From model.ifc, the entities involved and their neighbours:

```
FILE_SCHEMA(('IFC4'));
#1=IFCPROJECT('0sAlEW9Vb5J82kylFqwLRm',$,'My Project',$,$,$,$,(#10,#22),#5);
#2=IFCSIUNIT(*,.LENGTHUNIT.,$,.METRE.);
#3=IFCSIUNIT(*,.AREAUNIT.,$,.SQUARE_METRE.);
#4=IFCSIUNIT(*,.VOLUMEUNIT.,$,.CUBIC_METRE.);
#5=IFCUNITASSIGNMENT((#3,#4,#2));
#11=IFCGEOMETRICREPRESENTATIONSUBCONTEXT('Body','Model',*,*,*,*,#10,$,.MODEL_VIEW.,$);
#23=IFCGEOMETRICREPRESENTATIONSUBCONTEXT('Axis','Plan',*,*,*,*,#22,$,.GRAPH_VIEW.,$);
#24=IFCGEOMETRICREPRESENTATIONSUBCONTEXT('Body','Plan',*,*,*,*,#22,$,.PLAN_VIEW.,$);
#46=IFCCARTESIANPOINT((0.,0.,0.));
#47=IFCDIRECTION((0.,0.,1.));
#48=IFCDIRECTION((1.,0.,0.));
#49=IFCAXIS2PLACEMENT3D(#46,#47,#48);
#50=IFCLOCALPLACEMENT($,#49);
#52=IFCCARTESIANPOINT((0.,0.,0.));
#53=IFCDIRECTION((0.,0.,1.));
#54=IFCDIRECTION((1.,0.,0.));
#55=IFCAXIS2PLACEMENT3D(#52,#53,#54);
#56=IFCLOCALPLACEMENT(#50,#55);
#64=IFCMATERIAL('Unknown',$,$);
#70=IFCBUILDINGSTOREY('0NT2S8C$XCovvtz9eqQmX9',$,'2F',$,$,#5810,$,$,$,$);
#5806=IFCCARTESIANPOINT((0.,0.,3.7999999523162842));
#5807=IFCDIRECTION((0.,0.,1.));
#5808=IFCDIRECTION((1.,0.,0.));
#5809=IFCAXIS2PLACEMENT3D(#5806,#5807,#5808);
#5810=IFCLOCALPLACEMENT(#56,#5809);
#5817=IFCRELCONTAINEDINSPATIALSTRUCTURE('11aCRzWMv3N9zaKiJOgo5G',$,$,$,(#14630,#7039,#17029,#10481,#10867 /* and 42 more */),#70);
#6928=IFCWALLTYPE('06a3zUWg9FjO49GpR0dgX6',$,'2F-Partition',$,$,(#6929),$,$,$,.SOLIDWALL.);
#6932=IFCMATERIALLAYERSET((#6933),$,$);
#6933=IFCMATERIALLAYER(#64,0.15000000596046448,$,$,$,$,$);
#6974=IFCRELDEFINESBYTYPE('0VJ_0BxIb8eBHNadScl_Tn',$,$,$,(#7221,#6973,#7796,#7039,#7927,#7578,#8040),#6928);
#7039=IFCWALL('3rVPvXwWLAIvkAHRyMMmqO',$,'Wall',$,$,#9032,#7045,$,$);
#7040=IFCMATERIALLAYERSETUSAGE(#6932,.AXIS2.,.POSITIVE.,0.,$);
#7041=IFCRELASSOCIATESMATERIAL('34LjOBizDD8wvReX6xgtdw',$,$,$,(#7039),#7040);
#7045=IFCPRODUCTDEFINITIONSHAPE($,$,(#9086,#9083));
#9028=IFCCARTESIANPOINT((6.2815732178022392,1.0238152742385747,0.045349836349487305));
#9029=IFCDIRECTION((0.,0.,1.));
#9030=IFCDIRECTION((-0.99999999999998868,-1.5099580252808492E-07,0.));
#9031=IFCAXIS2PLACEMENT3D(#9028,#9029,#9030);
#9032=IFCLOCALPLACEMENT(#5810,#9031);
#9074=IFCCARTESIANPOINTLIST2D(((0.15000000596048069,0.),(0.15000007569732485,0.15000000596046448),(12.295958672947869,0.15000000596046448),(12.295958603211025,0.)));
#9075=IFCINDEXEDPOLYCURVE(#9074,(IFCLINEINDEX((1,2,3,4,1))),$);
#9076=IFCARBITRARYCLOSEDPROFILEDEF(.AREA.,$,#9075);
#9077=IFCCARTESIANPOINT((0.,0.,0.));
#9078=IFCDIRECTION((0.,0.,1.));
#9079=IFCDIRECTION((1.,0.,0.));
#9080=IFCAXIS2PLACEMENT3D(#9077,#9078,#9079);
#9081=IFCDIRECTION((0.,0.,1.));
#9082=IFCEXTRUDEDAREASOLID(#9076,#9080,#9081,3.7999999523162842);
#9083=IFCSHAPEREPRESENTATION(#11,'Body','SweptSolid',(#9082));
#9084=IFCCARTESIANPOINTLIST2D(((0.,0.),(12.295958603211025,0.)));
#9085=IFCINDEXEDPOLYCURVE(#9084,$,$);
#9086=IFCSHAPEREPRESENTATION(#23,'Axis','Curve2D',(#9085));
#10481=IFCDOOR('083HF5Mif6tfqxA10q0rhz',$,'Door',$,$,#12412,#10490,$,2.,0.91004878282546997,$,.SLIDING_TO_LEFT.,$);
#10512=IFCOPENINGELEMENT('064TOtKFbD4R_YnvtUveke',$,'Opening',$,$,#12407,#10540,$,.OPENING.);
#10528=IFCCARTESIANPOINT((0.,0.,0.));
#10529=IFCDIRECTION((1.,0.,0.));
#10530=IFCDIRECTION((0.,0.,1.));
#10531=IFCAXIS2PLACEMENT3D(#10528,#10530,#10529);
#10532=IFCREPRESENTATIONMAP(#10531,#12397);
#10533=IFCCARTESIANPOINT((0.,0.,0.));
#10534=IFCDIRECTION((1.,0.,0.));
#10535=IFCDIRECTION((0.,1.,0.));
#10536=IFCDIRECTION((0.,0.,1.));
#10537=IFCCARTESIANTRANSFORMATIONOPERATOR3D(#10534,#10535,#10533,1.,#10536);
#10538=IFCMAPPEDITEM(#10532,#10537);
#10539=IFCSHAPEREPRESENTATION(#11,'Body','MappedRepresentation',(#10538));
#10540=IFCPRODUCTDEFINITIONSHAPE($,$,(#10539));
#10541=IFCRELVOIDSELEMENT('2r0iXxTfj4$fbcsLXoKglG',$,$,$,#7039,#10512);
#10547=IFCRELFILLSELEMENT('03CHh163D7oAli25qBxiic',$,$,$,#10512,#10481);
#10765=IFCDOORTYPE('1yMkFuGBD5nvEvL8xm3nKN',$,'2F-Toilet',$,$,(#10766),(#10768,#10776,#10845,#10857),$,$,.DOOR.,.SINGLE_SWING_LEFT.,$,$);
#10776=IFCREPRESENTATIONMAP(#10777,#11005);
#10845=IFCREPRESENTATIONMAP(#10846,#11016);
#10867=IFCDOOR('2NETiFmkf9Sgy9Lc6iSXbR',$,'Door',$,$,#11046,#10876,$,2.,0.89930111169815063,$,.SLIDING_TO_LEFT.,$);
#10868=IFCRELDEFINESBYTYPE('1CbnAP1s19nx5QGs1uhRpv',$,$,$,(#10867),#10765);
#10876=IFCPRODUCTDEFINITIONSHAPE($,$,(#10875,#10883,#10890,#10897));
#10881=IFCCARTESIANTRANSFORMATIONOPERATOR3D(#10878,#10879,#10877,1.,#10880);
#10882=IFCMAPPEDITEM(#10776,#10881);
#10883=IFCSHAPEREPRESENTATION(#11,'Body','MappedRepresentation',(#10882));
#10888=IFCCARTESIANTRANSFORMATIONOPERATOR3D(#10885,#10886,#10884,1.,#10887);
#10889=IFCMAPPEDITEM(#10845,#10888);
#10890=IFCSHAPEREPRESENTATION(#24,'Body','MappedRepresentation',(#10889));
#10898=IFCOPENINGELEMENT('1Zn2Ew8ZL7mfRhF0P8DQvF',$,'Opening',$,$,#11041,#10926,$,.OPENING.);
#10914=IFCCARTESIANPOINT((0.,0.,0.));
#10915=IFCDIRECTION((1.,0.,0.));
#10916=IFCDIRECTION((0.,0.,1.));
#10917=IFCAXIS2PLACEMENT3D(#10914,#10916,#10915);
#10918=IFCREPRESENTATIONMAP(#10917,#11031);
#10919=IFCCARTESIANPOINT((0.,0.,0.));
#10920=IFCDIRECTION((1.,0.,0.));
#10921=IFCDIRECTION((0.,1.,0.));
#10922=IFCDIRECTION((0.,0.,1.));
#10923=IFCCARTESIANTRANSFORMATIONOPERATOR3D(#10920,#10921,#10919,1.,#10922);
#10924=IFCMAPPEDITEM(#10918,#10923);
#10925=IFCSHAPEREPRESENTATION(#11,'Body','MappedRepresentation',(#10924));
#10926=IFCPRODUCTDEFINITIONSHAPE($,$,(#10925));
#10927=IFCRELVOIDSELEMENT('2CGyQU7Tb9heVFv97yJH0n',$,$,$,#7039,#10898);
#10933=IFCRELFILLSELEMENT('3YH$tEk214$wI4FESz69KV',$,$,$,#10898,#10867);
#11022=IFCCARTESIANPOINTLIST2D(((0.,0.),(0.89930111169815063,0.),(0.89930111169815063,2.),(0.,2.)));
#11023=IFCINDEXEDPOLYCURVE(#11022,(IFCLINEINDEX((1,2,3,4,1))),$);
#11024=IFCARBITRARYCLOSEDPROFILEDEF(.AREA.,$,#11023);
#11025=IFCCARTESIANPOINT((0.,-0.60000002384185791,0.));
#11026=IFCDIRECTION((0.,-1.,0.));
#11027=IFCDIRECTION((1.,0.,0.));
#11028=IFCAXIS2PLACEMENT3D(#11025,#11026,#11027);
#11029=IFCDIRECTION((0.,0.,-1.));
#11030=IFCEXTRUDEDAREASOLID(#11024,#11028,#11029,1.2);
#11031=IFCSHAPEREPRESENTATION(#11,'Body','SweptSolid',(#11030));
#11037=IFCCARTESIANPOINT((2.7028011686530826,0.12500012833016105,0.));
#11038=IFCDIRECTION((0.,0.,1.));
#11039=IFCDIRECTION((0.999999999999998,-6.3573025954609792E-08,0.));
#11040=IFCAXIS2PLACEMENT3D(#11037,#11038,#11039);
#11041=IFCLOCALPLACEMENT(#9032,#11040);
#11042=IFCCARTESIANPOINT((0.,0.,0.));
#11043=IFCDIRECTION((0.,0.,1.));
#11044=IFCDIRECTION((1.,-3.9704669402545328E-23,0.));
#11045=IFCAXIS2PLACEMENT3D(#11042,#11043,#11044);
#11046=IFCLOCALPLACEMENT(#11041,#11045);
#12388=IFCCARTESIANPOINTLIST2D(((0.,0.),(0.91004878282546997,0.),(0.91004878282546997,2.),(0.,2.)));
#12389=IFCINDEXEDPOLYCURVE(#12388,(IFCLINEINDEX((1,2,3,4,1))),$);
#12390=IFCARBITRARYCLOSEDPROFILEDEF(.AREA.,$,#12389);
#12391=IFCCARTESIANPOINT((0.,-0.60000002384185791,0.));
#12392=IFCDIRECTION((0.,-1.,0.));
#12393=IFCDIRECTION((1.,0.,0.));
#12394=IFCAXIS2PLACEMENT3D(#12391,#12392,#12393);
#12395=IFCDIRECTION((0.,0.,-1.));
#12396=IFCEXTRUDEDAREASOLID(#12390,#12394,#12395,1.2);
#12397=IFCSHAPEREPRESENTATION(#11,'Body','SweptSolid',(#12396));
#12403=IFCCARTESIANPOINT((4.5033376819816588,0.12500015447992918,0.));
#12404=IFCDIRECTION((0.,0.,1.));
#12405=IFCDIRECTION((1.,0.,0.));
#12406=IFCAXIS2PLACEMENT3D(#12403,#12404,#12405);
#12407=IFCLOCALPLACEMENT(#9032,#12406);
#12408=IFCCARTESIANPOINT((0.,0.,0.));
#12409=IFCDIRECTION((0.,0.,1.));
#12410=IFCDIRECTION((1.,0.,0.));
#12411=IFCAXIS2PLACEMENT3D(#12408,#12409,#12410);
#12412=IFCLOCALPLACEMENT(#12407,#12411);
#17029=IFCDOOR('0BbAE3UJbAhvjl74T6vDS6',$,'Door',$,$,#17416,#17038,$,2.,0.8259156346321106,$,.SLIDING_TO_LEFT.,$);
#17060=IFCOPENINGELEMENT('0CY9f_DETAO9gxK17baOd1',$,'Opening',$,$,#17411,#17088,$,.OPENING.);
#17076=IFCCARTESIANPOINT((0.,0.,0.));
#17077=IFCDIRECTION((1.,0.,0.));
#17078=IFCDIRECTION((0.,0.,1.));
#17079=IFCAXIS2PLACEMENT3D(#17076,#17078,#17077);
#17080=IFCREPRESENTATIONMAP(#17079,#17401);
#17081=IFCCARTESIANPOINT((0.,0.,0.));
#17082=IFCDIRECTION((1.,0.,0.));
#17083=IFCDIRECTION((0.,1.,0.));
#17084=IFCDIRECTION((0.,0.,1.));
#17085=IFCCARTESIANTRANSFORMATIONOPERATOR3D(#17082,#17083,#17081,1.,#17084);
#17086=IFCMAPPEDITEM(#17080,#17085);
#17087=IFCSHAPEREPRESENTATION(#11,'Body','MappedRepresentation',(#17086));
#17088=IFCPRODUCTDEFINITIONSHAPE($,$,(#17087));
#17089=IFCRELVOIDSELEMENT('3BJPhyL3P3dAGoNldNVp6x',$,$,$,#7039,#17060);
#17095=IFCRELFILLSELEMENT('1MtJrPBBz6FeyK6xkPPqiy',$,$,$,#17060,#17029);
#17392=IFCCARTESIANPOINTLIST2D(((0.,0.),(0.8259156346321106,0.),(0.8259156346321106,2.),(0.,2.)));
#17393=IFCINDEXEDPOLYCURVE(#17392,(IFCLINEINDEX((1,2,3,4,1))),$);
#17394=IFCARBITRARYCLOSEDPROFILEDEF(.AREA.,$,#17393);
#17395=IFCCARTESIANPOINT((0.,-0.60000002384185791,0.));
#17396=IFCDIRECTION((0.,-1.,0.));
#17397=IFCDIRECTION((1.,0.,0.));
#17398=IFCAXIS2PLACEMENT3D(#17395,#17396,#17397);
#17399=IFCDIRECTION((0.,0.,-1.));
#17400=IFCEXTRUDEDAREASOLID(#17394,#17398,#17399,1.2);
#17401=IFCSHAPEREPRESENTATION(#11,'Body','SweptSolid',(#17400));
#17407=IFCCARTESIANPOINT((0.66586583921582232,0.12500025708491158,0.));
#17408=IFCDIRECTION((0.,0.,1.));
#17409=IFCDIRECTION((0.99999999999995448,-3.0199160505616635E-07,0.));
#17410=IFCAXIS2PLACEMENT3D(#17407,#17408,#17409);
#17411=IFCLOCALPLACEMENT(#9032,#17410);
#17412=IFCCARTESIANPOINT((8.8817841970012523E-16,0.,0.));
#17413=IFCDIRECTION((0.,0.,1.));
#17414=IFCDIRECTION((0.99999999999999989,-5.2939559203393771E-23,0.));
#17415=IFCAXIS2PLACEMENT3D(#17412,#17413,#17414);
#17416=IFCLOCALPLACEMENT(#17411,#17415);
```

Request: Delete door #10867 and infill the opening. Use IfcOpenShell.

```python
import ifcopenshell
import ifcopenshell.api.feature
import ifcopenshell.api.root
import ifcopenshell.geom
import ifcopenshell.util.shape

model = ifcopenshell.open("model.ifc")
settings = ifcopenshell.geom.settings()


def volume(element):
    """Net volume in cubic metres, openings subtracted."""
    shape = ifcopenshell.geom.create_shape(settings, element)
    return ifcopenshell.util.shape.get_volume(shape.geometry)


door = model.by_guid("2NETiFmkf9Sgy9Lc6iSXbR")
opening = door.FillsVoids[0].RelatingOpeningElement
wall = opening.VoidsElements[0].RelatingBuildingElement
before = volume(wall)

ifcopenshell.api.root.remove_product(model, product=door)
ifcopenshell.api.feature.remove_feature(model, feature=opening)

after = volume(wall)

print(f"wall volume {before:.3f} -> {after:.3f} m3")

model.write("model_rev.ifc")
```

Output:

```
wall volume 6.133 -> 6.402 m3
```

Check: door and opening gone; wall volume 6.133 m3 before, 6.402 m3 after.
